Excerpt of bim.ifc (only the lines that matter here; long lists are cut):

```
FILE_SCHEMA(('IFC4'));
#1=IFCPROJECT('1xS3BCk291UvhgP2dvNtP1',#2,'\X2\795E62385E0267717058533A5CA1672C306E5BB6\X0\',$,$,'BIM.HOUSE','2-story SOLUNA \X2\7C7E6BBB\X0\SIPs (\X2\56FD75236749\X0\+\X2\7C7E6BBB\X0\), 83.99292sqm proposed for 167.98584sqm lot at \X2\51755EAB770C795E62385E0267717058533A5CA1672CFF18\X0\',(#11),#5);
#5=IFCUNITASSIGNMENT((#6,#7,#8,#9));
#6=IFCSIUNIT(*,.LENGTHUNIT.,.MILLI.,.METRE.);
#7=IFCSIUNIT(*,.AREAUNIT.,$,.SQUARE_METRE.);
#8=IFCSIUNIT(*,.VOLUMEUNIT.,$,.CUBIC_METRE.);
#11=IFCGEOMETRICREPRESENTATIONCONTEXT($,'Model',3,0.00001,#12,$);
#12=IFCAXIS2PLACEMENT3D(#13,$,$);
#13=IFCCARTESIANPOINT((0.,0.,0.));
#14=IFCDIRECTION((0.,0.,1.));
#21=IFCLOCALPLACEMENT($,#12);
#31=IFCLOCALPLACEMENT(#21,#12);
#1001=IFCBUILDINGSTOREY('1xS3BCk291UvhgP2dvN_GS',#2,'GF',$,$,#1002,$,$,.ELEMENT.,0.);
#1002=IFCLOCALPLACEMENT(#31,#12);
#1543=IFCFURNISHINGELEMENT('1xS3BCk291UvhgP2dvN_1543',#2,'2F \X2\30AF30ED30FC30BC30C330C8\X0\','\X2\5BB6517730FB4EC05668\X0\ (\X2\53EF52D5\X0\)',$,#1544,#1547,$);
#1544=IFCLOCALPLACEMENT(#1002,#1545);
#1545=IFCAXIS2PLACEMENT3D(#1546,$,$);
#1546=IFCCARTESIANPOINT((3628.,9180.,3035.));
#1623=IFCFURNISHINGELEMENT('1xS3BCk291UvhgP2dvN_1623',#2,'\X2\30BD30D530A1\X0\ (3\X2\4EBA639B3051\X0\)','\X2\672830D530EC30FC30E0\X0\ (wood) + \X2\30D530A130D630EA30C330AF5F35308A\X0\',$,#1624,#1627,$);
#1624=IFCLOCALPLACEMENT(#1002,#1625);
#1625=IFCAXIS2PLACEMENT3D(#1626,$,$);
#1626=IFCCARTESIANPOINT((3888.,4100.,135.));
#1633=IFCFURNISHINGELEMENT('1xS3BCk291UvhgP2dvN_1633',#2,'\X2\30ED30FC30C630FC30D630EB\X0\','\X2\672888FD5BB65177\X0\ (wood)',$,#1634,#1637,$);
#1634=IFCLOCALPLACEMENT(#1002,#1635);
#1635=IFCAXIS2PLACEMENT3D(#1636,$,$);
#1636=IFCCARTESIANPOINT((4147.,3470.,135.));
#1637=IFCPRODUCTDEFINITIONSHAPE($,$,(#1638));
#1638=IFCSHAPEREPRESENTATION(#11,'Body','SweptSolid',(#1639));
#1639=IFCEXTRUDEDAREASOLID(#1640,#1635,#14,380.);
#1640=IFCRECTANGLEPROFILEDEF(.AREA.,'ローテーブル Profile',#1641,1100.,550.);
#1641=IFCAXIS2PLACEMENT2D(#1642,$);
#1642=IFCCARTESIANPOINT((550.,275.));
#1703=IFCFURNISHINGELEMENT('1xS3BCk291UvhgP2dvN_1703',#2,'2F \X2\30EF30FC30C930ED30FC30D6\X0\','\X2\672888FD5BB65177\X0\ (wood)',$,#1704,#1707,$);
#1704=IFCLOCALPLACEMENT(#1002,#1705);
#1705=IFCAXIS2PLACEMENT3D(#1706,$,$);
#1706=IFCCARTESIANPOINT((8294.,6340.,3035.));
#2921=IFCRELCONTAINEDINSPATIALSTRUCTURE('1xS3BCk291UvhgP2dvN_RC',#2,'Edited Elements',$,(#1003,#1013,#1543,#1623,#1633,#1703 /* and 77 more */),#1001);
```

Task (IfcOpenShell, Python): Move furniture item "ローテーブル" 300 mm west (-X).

```python
import ifcopenshell
import ifcopenshell.api.geometry
import ifcopenshell.util.placement
import ifcopenshell.util.unit

model = ifcopenshell.open("bim.ifc")
unit_scale = ifcopenshell.util.unit.calculate_unit_scale(model)

item = model.by_guid("1xS3BCk291UvhgP2dvN_1633")
matrix = ifcopenshell.util.placement.get_local_placement(item.ObjectPlacement)
matrix[0, 3] -= 0.3 / unit_scale
ifcopenshell.api.geometry.edit_object_placement(model, product=item, matrix=matrix, is_si=False)

print(ifcopenshell.util.placement.get_local_placement(item.ObjectPlacement).round(3) + 0.0)

model.write("bim_v2.ifc")
```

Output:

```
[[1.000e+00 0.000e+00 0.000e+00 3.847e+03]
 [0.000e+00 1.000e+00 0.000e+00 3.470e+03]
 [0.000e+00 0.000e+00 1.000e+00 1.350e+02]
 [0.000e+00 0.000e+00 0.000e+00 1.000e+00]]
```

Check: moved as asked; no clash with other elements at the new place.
